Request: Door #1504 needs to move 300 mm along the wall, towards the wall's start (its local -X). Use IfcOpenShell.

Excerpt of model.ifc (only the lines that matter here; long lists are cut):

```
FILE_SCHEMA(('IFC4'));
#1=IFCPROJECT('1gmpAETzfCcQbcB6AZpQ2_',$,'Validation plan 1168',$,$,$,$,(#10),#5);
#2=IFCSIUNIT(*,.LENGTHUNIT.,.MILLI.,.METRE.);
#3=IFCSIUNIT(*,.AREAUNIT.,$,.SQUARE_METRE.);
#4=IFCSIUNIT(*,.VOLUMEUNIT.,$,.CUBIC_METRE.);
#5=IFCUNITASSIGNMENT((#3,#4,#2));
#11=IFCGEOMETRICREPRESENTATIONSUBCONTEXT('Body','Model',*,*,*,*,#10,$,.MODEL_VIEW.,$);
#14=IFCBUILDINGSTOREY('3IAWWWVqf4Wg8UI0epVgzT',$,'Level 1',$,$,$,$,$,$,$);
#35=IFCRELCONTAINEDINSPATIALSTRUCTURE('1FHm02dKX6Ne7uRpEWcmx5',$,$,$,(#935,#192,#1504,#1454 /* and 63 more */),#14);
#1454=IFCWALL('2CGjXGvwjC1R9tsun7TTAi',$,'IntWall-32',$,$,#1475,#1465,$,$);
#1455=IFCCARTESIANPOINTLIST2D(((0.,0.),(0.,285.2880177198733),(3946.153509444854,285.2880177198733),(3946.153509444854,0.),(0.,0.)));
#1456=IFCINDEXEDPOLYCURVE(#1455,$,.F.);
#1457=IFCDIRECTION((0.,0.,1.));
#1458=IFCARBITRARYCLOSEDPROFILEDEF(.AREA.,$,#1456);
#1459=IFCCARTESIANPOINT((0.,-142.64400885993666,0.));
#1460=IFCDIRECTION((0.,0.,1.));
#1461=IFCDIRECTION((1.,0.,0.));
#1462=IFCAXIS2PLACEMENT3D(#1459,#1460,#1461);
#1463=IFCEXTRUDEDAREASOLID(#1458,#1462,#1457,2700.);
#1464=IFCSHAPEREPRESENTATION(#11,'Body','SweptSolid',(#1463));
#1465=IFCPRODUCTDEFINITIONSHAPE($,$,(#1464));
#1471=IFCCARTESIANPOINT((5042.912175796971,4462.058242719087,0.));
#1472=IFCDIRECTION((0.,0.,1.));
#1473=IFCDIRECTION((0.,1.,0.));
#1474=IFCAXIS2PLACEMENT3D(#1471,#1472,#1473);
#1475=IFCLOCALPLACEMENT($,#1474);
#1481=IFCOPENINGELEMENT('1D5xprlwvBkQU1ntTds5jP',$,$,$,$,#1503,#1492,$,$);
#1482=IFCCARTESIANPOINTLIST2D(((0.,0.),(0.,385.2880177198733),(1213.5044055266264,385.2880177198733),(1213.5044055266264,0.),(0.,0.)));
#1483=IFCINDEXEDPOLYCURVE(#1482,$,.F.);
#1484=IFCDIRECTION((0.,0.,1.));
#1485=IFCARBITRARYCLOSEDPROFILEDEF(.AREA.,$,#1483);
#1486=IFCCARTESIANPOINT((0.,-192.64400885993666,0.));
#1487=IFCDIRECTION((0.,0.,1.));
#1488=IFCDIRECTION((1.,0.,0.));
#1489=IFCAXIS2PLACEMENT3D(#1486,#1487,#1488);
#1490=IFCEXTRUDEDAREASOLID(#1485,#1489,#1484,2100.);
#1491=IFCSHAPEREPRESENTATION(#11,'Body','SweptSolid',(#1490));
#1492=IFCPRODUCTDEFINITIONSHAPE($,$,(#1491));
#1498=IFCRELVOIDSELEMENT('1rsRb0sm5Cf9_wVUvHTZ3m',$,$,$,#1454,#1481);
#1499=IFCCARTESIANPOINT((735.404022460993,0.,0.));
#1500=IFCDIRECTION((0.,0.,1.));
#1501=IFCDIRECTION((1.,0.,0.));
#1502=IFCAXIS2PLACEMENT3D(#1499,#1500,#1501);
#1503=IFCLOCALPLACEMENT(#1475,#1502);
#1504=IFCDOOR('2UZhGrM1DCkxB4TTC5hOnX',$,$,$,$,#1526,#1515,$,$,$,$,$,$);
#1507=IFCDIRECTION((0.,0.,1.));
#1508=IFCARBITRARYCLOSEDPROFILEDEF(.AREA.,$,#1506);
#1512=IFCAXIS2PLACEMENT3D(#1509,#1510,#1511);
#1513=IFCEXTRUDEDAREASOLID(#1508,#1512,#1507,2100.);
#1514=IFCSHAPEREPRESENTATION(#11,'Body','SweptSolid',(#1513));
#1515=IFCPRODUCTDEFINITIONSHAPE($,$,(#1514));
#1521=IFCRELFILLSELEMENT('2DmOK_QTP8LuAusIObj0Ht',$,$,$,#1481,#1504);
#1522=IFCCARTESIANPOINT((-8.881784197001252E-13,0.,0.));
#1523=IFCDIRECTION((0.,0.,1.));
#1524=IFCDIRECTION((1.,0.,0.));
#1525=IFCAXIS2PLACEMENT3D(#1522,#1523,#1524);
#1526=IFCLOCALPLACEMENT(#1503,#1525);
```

```python
import ifcopenshell
import ifcopenshell.api.geometry
import ifcopenshell.util.placement
import ifcopenshell.util.unit

model = ifcopenshell.open("model.ifc")
unit_scale = ifcopenshell.util.unit.calculate_unit_scale(model)

door = model.by_guid("2UZhGrM1DCkxB4TTC5hOnX")
opening = door.FillsVoids[0].RelatingOpeningElement
wall = opening.VoidsElements[0].RelatingBuildingElement

wall_matrix = ifcopenshell.util.placement.get_local_placement(wall.ObjectPlacement)
shift = wall_matrix[:3, 0] * -0.3 / unit_scale
before = ifcopenshell.util.placement.get_local_placement(door.ObjectPlacement)[:3, 3].copy()

# The door is placed relative to its opening, so it follows when the opening moves.
matrix = ifcopenshell.util.placement.get_local_placement(opening.ObjectPlacement)
matrix[:3, 3] += shift
ifcopenshell.api.geometry.edit_object_placement(
    model, product=opening, matrix=matrix, is_si=False, should_transform_children=True
)

after = ifcopenshell.util.placement.get_local_placement(door.ObjectPlacement)[:3, 3]
print("door moved by", (after - before).round(3) + 0.0)

model.write("model_edited.ifc")
```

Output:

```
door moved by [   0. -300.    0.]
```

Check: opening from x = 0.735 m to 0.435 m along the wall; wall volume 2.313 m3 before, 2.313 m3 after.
